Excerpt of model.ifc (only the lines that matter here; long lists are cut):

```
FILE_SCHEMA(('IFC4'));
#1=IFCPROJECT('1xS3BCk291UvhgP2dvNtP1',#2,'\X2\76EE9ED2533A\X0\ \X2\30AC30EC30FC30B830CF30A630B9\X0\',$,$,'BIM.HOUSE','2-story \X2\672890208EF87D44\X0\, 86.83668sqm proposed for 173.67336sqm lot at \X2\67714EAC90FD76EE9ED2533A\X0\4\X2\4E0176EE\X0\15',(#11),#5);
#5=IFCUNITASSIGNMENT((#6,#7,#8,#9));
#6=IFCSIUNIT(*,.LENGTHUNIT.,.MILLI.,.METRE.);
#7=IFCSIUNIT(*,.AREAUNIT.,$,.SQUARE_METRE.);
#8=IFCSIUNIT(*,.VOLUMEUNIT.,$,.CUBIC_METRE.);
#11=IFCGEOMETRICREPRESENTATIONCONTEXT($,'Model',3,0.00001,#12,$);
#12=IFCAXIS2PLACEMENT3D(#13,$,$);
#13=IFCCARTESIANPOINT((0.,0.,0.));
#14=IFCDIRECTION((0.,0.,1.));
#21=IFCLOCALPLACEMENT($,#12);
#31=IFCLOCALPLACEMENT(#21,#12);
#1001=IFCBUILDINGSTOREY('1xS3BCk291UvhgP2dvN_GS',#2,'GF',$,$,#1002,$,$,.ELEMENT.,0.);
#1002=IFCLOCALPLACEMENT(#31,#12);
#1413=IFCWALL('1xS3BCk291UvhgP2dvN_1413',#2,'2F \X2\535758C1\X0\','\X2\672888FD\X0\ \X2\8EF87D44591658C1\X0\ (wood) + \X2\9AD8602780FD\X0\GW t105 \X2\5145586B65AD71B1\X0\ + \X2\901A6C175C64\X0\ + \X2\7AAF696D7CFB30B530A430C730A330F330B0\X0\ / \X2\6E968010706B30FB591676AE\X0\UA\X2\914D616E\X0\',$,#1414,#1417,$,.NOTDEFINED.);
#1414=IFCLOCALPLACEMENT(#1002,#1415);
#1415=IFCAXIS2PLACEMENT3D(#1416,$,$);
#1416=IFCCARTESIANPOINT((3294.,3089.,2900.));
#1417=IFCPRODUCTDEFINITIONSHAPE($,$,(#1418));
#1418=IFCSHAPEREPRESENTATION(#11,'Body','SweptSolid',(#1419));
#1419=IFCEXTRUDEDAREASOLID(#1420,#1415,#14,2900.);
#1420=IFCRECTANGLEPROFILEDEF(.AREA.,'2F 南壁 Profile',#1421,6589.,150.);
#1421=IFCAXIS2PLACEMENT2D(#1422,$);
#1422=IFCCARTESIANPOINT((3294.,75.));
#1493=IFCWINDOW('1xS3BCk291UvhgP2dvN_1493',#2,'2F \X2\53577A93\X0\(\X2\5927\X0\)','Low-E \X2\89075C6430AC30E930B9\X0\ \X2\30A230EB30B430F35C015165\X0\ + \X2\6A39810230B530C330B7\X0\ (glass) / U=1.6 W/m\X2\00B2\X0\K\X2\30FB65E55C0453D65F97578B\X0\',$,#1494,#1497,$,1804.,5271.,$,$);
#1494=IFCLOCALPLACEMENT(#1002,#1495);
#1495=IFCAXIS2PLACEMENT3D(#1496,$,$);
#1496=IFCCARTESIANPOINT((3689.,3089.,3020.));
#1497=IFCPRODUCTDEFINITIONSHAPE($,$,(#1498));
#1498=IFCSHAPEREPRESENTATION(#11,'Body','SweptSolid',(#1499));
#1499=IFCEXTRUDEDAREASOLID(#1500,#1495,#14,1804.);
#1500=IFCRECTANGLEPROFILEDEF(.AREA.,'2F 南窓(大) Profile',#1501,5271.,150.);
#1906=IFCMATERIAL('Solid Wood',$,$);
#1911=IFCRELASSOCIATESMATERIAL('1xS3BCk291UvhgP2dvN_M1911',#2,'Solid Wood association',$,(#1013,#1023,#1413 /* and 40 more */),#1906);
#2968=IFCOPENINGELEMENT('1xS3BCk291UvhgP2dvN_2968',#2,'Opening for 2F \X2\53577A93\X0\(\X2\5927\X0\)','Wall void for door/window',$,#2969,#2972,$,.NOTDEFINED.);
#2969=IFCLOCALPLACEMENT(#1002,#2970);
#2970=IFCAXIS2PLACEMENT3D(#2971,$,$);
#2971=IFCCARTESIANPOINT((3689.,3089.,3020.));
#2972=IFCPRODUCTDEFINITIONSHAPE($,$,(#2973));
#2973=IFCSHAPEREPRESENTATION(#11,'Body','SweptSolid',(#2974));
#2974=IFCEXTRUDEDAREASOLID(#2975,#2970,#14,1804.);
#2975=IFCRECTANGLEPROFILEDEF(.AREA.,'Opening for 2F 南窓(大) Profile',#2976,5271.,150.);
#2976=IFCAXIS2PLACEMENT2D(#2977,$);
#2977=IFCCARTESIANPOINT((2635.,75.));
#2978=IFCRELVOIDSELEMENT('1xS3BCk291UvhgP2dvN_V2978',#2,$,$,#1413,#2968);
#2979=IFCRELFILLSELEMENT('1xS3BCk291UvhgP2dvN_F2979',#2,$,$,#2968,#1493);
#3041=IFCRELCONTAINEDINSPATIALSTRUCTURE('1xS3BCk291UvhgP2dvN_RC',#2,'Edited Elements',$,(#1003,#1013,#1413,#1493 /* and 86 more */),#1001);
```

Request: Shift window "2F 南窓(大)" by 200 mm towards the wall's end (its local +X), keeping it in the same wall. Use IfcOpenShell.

```python
import ifcopenshell
import ifcopenshell.api.geometry
import ifcopenshell.util.placement
import ifcopenshell.util.unit

model = ifcopenshell.open("model.ifc")
unit_scale = ifcopenshell.util.unit.calculate_unit_scale(model)

window = model.by_guid("1xS3BCk291UvhgP2dvN_1493")
opening = window.FillsVoids[0].RelatingOpeningElement
wall = opening.VoidsElements[0].RelatingBuildingElement

wall_matrix = ifcopenshell.util.placement.get_local_placement(wall.ObjectPlacement)
shift = wall_matrix[:3, 0] * 0.2 / unit_scale
before = ifcopenshell.util.placement.get_local_placement(window.ObjectPlacement)[:3, 3].copy()

# The window is not placed relative to its opening, so move both.
for product in (opening, window):
    matrix = ifcopenshell.util.placement.get_local_placement(product.ObjectPlacement)
    matrix[:3, 3] += shift
    ifcopenshell.api.geometry.edit_object_placement(model, product=product, matrix=matrix, is_si=False)

after = ifcopenshell.util.placement.get_local_placement(window.ObjectPlacement)[:3, 3]
print("window moved by", (after - before).round(3) + 0.0)

model.write("model_v2.ifc")
```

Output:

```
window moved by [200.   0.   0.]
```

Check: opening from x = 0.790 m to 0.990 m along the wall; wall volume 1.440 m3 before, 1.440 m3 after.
